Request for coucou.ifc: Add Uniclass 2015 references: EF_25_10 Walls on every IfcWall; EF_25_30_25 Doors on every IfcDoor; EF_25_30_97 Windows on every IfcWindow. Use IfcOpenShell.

First a look at what the model holds.

```python
import ifcopenshell

model = ifcopenshell.open("coucou.ifc")
print(model.schema)
print("classifications:", [c.Name for c in model.by_type("IfcClassification")])
for ifc_class in ("IfcDoor", "IfcRoof", "IfcStair", "IfcWall", "IfcWindow"):
    print(ifc_class, len(model.by_type(ifc_class)))
```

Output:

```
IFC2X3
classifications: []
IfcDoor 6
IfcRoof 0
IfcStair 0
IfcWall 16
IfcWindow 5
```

```python
import ifcopenshell
import ifcopenshell.api.classification

model = ifcopenshell.open("coucou.ifc")

# IFC2X3 requires Source and Edition and has no link from the project to the system.
system = model.create_entity("IfcClassification", Source="NBS", Edition="2015", Name="Uniclass 2015")

codes = {
    "IfcWall": ("EF_25_10", "Walls"),
    "IfcDoor": ("EF_25_30_25", "Doors"),
    "IfcWindow": ("EF_25_30_97", "Windows"),
}
for ifc_class, (code, name) in codes.items():
    products = model.by_type(ifc_class)
    ifcopenshell.api.classification.add_reference(
        model, products=products, classification=system, identification=code, name=name
    )
    print(code, len(products))

model.write("coucou_rev.ifc")
```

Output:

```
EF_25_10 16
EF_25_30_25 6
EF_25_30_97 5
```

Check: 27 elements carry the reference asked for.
